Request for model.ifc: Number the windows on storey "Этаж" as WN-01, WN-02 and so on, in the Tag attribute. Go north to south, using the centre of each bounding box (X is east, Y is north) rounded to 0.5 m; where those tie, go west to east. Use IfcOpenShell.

First a look at what the model holds.

```python
import ifcopenshell
import ifcopenshell.util.element
import ifcopenshell.util.placement

model = ifcopenshell.open("model.ifc")
print(model.schema)
storey = next(s for s in model.by_type("IfcBuildingStorey") if s.Name == "Этаж")
windows = [e for e in ifcopenshell.util.element.get_decomposition(storey) if e.is_a("IfcWindow")]
for e in sorted(windows, key=lambda e: e.id()):
    origin = ifcopenshell.util.placement.get_local_placement(e.ObjectPlacement)[:3, 3]
    print(e.id(), e.Tag, e.Name, origin.round(2) + 0.0, sep=" | ")
```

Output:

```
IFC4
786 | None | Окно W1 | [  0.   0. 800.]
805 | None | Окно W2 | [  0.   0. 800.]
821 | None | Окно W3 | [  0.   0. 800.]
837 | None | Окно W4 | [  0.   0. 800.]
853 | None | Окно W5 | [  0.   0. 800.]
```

```python
import ifcopenshell
import ifcopenshell.geom
import ifcopenshell.util.element
import ifcopenshell.util.shape

model = ifcopenshell.open("model.ifc")
settings = ifcopenshell.geom.settings()
settings.set("use-world-coords", True)


def centre(element):
    shape = ifcopenshell.geom.create_shape(settings, element)
    return ifcopenshell.util.shape.get_bbox_centroid(shape.geometry)


storey = next(s for s in model.by_type("IfcBuildingStorey") if s.Name == "Этаж")
windows = [e for e in ifcopenshell.util.element.get_decomposition(storey) if e.is_a("IfcWindow")]

# Insertion points can sit at a corner or the storey origin, so sort by the geometry (in metres).
centres = {e: centre(e) for e in windows}
windows.sort(key=lambda e: (-round(centres[e][1] / 0.5), centres[e][0]))

for i, e in enumerate(windows, start=1):
    number = f"WN-{i:02d}"
    e.Tag = number
    print(e.id(), number)

model.write("model_rev.ifc")
```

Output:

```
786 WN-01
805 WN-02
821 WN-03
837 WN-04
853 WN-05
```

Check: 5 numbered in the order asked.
